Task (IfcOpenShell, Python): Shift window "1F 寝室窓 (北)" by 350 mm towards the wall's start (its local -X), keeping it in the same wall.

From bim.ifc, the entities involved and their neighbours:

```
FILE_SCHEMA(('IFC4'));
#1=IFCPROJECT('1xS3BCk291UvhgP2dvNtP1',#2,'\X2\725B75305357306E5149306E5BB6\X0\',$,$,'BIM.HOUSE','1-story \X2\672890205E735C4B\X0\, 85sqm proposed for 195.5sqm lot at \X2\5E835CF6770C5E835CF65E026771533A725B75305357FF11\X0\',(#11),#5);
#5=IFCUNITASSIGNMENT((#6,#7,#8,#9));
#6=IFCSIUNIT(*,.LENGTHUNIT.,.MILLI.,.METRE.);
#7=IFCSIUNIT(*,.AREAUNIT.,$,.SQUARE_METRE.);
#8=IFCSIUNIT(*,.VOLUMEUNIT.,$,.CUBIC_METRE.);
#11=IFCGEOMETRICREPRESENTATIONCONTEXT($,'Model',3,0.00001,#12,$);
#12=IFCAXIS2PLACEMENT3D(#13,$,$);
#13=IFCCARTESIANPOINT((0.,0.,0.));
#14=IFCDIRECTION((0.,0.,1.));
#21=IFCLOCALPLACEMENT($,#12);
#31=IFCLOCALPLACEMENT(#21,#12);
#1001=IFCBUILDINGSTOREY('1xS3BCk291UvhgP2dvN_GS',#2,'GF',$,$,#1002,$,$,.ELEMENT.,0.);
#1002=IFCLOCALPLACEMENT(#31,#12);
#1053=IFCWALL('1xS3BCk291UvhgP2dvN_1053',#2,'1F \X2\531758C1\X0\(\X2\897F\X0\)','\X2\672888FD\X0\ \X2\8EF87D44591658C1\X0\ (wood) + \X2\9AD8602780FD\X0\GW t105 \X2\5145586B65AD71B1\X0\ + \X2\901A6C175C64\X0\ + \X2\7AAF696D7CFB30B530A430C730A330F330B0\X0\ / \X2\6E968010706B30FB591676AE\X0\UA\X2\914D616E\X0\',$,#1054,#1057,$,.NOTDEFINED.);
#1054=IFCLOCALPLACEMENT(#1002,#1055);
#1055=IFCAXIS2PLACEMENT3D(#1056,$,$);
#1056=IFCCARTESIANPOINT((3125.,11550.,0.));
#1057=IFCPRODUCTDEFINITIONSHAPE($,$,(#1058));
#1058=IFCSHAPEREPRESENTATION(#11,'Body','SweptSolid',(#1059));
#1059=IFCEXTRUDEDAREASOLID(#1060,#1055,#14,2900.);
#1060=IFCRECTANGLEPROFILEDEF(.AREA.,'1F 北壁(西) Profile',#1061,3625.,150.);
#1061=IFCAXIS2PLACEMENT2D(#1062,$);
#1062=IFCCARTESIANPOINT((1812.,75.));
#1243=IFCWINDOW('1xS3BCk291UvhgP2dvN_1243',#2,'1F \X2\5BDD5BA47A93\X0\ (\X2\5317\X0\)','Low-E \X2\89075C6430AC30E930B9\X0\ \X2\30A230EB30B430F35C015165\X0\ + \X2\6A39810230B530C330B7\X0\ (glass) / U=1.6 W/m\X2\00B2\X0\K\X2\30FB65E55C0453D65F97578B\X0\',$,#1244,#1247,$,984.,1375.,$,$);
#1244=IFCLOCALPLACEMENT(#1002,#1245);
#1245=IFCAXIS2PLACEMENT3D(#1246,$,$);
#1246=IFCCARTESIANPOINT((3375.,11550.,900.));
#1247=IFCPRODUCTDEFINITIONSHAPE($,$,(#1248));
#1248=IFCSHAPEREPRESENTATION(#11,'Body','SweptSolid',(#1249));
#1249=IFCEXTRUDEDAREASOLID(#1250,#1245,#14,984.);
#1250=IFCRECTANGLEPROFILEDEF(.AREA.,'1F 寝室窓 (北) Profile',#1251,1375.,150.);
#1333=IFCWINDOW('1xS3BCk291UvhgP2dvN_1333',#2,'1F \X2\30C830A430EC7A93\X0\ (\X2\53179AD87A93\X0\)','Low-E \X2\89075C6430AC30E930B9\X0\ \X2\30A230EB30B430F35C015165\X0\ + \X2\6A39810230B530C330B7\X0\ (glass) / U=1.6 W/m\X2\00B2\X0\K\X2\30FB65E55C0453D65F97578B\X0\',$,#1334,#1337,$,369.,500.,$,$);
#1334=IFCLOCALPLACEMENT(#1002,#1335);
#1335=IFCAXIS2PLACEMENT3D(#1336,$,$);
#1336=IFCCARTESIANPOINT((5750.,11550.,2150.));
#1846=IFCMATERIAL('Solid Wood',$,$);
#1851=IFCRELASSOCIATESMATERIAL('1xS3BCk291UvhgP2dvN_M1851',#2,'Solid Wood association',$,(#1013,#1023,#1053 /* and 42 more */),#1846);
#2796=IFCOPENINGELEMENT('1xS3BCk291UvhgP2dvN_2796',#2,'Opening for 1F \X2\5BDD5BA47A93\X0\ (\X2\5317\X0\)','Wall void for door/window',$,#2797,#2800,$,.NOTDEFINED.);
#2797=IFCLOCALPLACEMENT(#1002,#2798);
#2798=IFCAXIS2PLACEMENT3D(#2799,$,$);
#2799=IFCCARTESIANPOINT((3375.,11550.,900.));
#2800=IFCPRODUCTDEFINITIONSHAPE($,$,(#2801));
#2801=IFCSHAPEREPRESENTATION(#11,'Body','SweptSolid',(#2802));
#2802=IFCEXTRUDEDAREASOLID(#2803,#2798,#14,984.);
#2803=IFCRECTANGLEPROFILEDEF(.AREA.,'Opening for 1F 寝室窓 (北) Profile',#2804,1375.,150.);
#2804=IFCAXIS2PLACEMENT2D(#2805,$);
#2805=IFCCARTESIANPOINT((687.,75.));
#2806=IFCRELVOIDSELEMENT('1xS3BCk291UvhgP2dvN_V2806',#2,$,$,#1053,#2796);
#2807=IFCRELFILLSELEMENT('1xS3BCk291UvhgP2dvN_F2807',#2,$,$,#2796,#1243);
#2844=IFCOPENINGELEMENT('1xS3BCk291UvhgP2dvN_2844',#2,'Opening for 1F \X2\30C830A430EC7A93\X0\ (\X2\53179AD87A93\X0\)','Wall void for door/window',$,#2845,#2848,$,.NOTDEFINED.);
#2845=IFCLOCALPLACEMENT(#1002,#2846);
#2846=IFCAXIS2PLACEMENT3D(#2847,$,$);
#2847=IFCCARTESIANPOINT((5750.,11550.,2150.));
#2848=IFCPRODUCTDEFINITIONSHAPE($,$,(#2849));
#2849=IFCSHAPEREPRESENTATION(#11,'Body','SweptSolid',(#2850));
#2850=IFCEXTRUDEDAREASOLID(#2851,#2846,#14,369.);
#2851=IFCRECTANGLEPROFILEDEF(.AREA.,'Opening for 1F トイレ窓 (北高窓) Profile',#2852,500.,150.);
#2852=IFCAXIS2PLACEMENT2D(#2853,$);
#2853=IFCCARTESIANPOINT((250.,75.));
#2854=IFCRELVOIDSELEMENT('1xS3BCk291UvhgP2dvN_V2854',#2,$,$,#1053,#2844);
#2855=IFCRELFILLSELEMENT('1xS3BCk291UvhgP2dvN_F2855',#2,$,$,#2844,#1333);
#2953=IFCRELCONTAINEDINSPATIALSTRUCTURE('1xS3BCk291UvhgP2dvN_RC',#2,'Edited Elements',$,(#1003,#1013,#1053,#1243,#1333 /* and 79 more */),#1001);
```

```python
import ifcopenshell
import ifcopenshell.api.geometry
import ifcopenshell.util.placement
import ifcopenshell.util.unit

model = ifcopenshell.open("bim.ifc")
unit_scale = ifcopenshell.util.unit.calculate_unit_scale(model)

window = model.by_guid("1xS3BCk291UvhgP2dvN_1243")
opening = window.FillsVoids[0].RelatingOpeningElement
wall = opening.VoidsElements[0].RelatingBuildingElement

wall_matrix = ifcopenshell.util.placement.get_local_placement(wall.ObjectPlacement)
shift = wall_matrix[:3, 0] * -0.35 / unit_scale
before = ifcopenshell.util.placement.get_local_placement(window.ObjectPlacement)[:3, 3].copy()

# The window is not placed relative to its opening, so move both.
for product in (opening, window):
    matrix = ifcopenshell.util.placement.get_local_placement(product.ObjectPlacement)
    matrix[:3, 3] += shift
    ifcopenshell.api.geometry.edit_object_placement(model, product=product, matrix=matrix, is_si=False)

after = ifcopenshell.util.placement.get_local_placement(window.ObjectPlacement)[:3, 3]
print("window moved by", (after - before).round(3) + 0.0)

model.write("bim_rev.ifc")
```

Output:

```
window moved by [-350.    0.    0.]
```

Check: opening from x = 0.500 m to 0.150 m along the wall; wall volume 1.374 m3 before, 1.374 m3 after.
